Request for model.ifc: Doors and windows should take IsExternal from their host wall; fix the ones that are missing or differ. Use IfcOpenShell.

First a look at what the model holds.

```python
import ifcopenshell
import ifcopenshell.util.element

model = ifcopenshell.open("model.ifc")
print(model.schema)
seen = {}
for e in model.by_type("IfcDoor") + model.by_type("IfcWindow"):
    if not e.FillsVoids:
        continue
    host = e.FillsVoids[0].RelatingOpeningElement.VoidsElements[0].RelatingBuildingElement
    own = ifcopenshell.util.element.get_pset(e, f"Pset_{e.is_a()[3:].removesuffix('StandardCase')}Common", "IsExternal")
    wall = ifcopenshell.util.element.get_pset(host, "Pset_WallCommon", "IsExternal")
    seen[e.is_a(), own, wall] = seen.get((e.is_a(), own, wall), 0) + 1
for (cls, own, wall), count in sorted(seen.items(), key=str):
    print(count, cls, "IsExternal:", own, "| host wall:", wall)
```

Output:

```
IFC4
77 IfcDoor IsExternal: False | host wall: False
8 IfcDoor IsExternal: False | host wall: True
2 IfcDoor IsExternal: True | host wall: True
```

```python
import ifcopenshell
import ifcopenshell.api.pset
import ifcopenshell.util.element

model = ifcopenshell.open("model.ifc")

count = 0
for ifc_class, pset_name in (("IfcDoor", "Pset_DoorCommon"), ("IfcWindow", "Pset_WindowCommon")):
    for e in model.by_type(ifc_class):
        if not e.FillsVoids:
            continue
        host = e.FillsVoids[0].RelatingOpeningElement.VoidsElements[0].RelatingBuildingElement
        external = ifcopenshell.util.element.get_pset(host, "Pset_WallCommon", "IsExternal")
        if external is None or ifcopenshell.util.element.get_pset(e, pset_name, "IsExternal") == external:
            continue
        pset = ifcopenshell.api.pset.add_pset(model, product=e, name=pset_name)
        ifcopenshell.api.pset.edit_pset(model, pset=pset, properties={"IsExternal": external})
        count += 1

print(count, "updated")

model.write("model_rev.ifc")
```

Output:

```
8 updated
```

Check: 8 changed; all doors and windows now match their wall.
